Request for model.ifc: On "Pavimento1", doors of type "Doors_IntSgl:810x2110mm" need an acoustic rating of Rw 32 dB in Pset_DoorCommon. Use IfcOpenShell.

First a look at what the model holds.

```python
import ifcopenshell
import ifcopenshell.util.element

model = ifcopenshell.open("model.ifc")
print(model.schema)
storey = next(s for s in model.by_type("IfcBuildingStorey") if s.Name == "Pavimento1")
doors = [e for e in ifcopenshell.util.element.get_decomposition(storey) if e.is_a("IfcDoor")]
seen = {}
for e in doors:
    element_type = ifcopenshell.util.element.get_type(e)
    key = (element_type.Name if element_type != e and element_type else None, ifcopenshell.util.element.get_pset(e, "Pset_DoorCommon", "AcousticRating"))
    seen[key] = seen.get(key, 0) + 1
for (name, value), count in sorted(seen.items(), key=str):
    print(count, "x", name, "|", value)
```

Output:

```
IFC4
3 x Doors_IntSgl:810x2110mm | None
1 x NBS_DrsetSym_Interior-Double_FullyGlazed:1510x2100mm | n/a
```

```python
import ifcopenshell
import ifcopenshell.api.pset
import ifcopenshell.util.element

model = ifcopenshell.open("model.ifc")

storey = next(s for s in model.by_type("IfcBuildingStorey") if s.Name == "Pavimento1")
doors = [e for e in ifcopenshell.util.element.get_decomposition(storey) if e.is_a("IfcDoor")]

count = 0
for e in doors:
    element_type = ifcopenshell.util.element.get_type(e)
    if element_type in (None, e) or element_type.Name != "Doors_IntSgl:810x2110mm":
        continue
    # add_pset returns the element's existing set when there is one.
    pset = ifcopenshell.api.pset.add_pset(model, product=e, name="Pset_DoorCommon")
    ifcopenshell.api.pset.edit_pset(model, pset=pset, properties={"AcousticRating": "Rw 32 dB"})
    count += 1

print(count, "doors updated")

model.write("model_rev.ifc")
```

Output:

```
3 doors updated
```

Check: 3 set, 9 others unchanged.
